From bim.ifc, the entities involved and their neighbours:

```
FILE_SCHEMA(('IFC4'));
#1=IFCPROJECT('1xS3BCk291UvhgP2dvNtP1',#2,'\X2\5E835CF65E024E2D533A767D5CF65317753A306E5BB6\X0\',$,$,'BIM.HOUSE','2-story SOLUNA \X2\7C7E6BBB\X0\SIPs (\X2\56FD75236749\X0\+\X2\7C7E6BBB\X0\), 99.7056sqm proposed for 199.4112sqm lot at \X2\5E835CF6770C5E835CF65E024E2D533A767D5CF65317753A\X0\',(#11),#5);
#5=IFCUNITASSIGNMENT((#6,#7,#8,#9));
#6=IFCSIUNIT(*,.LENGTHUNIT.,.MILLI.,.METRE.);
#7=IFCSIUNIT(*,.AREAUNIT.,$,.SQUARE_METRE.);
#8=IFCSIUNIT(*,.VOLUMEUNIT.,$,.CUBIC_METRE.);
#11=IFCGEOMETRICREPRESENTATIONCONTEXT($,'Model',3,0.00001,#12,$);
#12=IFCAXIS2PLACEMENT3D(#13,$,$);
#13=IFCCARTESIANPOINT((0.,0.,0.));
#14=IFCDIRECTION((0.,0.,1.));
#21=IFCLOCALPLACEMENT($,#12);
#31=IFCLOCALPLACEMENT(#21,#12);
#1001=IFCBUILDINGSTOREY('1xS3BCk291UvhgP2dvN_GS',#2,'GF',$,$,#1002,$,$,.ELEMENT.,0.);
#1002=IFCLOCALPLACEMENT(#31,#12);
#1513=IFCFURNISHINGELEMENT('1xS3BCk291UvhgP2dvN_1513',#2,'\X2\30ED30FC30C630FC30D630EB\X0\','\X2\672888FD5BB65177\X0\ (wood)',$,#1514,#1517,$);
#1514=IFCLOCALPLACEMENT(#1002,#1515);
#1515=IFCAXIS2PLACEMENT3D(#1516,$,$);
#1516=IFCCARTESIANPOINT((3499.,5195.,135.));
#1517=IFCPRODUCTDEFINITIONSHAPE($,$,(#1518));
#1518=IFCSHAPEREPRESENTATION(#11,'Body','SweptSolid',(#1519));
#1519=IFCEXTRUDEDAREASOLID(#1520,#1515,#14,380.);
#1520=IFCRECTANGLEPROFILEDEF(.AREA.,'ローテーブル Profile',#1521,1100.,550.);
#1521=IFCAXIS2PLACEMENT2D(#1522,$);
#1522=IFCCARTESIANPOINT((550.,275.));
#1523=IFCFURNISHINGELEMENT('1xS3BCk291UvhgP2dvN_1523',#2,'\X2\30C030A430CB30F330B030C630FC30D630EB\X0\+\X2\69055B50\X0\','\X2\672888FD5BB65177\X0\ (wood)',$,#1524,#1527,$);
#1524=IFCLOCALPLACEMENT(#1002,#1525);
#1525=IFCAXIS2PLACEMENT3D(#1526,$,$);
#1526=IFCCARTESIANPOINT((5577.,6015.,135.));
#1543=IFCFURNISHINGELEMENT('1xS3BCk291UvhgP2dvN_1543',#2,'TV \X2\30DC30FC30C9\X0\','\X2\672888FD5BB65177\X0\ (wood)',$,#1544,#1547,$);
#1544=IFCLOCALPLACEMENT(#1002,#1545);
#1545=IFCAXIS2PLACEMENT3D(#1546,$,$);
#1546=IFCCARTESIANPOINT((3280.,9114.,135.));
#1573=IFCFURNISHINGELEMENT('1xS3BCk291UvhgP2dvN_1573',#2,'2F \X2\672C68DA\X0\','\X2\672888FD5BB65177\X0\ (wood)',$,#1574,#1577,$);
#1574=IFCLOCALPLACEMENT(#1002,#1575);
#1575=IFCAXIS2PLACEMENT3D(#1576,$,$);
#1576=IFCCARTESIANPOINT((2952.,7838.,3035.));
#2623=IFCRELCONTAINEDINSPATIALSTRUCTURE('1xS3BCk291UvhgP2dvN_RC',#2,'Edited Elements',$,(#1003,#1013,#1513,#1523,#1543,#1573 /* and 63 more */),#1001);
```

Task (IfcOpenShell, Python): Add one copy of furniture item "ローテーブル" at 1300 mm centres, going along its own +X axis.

```python
import ifcopenshell
import ifcopenshell.api.geometry
import ifcopenshell.api.root
import ifcopenshell.util.element
import ifcopenshell.util.placement
import ifcopenshell.util.unit

model = ifcopenshell.open("bim.ifc")
unit_scale = ifcopenshell.util.unit.calculate_unit_scale(model)


def reuse_history(source, copy):
    """copy_class also copies each property set's owner history, people and application; keep the originals."""
    for rel in copy.IsDefinedBy:
        if rel.is_a("IfcRelDefinesByProperties") and (history := rel.RelatingPropertyDefinition.OwnerHistory):
            rel.RelatingPropertyDefinition.OwnerHistory = source.OwnerHistory
            ifcopenshell.util.element.remove_deep2(model, history)


source = model.by_guid("1xS3BCk291UvhgP2dvN_1513")
base = ifcopenshell.util.placement.get_local_placement(source.ObjectPlacement)
step = base[:3, 0] * 1.3 / unit_scale

for i in range(1, 2):
    copy = ifcopenshell.api.root.copy_class(model, product=source)
    copy.Representation = ifcopenshell.util.element.copy_deep(
        model, source.Representation, exclude=["IfcGeometricRepresentationContext", "IfcRepresentationMap"]
    )
    reuse_history(source, copy)
    matrix = base.copy()
    matrix[:3, 3] += i * step
    print("added at", matrix[:3, 3].round(3) + 0.0)
    ifcopenshell.api.geometry.edit_object_placement(model, product=copy, matrix=matrix, is_si=False)

model.write("bim_v2.ifc")
```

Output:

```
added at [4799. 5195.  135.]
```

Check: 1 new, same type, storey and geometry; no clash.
